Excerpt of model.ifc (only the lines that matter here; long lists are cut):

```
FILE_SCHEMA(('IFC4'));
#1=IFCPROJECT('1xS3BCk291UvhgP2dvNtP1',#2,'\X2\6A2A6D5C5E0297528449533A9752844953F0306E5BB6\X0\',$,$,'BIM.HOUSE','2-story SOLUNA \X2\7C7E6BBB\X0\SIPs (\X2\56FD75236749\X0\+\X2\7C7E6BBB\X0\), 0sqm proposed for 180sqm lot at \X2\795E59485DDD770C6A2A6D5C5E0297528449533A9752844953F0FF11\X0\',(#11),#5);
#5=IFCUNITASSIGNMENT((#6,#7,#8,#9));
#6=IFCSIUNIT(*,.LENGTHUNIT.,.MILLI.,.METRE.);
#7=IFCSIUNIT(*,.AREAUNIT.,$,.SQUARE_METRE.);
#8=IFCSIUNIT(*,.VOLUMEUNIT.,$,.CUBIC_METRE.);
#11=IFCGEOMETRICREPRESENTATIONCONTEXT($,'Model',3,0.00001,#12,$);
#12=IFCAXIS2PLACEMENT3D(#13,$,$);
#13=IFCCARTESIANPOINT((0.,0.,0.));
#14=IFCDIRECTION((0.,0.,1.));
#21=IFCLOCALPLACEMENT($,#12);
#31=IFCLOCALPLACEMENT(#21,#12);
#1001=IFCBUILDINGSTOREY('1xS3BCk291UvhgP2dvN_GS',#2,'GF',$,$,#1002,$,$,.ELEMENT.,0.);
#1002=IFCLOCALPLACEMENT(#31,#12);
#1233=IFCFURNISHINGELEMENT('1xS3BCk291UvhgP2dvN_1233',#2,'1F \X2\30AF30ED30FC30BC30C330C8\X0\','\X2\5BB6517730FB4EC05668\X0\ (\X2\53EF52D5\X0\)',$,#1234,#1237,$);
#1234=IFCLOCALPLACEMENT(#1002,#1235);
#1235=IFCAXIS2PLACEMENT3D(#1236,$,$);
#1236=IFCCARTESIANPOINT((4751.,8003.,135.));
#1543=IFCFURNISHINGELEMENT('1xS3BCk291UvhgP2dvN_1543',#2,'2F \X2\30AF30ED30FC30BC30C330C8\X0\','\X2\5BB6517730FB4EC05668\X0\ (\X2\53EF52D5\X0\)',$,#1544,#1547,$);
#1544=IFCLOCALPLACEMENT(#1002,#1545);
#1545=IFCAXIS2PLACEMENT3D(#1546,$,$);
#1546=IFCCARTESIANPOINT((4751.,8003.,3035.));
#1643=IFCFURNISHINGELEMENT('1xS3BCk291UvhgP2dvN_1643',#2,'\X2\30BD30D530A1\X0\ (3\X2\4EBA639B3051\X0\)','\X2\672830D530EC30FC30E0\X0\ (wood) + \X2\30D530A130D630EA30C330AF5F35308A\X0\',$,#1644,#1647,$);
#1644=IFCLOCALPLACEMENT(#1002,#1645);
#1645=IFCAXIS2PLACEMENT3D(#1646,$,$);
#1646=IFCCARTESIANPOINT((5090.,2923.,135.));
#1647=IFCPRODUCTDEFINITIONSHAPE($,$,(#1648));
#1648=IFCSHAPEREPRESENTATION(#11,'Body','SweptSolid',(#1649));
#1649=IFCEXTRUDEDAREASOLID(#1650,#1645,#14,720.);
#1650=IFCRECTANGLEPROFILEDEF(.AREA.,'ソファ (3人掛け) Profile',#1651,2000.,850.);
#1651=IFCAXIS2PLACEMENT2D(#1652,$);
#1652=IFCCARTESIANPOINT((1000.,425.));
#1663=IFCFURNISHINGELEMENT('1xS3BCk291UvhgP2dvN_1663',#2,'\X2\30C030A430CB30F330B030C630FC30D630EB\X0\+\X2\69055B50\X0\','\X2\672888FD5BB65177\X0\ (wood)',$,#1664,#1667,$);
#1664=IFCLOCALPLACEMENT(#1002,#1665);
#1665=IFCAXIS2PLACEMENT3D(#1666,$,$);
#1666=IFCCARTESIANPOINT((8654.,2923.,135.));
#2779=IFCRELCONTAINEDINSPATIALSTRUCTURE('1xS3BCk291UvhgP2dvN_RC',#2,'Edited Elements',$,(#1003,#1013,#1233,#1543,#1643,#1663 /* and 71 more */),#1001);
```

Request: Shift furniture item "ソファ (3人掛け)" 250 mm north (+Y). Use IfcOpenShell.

```python
import ifcopenshell
import ifcopenshell.api.geometry
import ifcopenshell.util.placement

model = ifcopenshell.open("model.ifc")

item = model.by_id(1643)
matrix = ifcopenshell.util.placement.get_local_placement(item.ObjectPlacement)
matrix[1, 3] += 250.0
ifcopenshell.api.geometry.edit_object_placement(model, product=item, matrix=matrix, is_si=False)

print(ifcopenshell.util.placement.get_local_placement(item.ObjectPlacement).round(3) + 0.0)

model.write("model_rev.ifc")
```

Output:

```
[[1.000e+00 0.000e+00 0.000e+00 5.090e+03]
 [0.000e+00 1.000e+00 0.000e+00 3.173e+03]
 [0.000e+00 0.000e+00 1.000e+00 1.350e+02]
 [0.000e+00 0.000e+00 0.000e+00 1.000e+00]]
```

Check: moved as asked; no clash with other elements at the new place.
